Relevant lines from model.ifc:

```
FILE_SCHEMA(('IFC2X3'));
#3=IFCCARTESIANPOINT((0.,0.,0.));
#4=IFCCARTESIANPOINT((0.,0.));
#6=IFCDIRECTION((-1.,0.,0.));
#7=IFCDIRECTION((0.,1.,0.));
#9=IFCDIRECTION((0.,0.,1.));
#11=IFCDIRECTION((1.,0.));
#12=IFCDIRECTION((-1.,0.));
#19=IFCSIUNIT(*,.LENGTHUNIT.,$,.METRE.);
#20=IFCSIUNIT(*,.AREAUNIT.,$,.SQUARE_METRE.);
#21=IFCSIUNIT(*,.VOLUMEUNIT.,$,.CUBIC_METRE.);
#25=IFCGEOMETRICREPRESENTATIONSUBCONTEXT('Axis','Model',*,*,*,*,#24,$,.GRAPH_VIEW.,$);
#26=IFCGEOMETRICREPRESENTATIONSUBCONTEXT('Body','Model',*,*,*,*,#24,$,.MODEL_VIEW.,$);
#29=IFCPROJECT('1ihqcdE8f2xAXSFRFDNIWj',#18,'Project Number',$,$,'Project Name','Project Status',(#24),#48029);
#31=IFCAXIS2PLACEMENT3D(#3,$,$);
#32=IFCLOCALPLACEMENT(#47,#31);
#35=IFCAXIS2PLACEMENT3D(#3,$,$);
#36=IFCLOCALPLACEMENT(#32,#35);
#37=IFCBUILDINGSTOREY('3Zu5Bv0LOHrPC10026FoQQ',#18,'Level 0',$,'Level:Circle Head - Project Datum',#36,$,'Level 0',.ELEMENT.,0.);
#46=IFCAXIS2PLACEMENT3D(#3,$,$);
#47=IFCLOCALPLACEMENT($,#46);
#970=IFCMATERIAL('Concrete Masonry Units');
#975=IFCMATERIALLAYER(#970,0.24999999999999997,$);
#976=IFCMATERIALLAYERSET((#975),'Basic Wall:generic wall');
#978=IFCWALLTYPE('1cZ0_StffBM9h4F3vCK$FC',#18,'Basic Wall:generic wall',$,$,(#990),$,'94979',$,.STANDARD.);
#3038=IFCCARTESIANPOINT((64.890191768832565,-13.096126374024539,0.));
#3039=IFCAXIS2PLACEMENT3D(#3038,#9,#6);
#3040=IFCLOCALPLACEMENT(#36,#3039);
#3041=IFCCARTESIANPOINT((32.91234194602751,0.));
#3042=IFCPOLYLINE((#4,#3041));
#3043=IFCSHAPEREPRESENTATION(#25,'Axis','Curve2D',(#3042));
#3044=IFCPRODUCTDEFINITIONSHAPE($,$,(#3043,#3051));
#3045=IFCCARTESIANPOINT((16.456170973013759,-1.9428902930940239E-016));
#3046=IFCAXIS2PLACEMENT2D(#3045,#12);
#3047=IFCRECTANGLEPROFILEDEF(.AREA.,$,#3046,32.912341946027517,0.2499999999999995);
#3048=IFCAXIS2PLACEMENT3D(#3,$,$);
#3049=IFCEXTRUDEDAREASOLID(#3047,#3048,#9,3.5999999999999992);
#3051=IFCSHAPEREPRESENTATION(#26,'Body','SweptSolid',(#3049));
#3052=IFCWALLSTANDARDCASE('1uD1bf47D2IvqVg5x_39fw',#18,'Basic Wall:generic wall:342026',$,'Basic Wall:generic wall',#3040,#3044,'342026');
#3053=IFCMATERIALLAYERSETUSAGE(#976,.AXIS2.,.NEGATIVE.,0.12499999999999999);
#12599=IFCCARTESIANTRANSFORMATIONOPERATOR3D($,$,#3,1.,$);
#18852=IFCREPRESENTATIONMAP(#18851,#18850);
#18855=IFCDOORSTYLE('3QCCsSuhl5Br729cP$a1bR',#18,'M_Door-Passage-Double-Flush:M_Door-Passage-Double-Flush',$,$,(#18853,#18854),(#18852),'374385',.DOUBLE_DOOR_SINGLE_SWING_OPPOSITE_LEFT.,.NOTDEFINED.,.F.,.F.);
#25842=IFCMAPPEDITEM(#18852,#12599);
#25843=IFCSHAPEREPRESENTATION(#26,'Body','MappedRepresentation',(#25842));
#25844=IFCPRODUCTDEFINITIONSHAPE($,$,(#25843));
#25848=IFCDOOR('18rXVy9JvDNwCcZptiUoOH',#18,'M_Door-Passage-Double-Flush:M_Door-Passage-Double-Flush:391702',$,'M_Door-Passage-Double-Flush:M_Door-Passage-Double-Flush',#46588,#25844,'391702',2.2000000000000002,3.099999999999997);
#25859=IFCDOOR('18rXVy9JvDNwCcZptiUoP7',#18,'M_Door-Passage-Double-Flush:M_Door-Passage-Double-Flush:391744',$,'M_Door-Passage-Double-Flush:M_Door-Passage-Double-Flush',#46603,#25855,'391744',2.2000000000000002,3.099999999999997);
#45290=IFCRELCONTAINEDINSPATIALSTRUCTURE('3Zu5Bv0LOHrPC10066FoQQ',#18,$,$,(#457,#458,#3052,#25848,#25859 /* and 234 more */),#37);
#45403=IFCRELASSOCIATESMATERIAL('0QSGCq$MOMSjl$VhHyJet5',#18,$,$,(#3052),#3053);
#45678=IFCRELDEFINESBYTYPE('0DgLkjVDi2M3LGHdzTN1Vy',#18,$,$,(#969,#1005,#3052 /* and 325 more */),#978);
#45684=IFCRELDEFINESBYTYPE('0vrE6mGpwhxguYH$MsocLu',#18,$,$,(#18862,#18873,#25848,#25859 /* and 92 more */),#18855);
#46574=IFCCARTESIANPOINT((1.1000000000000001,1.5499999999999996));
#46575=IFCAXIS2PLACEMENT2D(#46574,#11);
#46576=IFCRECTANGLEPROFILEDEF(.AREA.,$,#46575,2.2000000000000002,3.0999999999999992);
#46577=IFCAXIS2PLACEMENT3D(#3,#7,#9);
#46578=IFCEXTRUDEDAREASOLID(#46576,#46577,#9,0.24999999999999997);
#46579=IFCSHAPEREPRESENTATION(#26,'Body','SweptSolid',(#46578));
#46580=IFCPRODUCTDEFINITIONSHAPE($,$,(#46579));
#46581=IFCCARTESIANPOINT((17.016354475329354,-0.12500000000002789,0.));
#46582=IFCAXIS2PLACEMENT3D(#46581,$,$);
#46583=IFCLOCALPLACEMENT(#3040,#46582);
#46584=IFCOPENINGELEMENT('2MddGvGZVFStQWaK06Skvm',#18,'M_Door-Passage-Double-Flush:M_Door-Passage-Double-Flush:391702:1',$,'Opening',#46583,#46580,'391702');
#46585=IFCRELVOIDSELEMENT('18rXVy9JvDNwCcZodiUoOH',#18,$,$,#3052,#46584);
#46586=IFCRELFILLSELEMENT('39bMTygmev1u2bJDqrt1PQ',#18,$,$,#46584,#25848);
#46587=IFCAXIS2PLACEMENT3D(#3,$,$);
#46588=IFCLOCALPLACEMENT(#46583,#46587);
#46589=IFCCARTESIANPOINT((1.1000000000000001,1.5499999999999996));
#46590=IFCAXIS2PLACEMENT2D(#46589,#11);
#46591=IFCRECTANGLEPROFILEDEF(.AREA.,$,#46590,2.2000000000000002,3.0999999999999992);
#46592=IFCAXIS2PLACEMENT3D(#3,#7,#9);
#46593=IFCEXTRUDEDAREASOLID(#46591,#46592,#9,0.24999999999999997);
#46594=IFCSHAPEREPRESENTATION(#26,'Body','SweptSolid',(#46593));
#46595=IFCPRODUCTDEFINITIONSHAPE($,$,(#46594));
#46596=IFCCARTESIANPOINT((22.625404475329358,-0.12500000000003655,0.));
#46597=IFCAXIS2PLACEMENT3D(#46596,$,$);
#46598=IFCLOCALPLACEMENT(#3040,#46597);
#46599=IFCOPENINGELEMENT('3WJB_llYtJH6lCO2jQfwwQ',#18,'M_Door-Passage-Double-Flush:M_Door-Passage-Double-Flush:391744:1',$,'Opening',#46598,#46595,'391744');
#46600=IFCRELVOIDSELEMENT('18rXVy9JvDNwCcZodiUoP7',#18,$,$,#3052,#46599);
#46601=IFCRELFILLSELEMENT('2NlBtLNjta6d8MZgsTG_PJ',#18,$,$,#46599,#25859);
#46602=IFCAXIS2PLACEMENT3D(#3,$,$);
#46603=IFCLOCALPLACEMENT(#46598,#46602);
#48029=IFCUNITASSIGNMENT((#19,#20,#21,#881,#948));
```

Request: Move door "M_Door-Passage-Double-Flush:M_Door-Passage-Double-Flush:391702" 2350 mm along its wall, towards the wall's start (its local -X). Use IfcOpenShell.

```python
import ifcopenshell
import ifcopenshell.api.geometry
import ifcopenshell.util.placement
import ifcopenshell.util.unit

model = ifcopenshell.open("model.ifc")
unit_scale = ifcopenshell.util.unit.calculate_unit_scale(model)

door = model.by_guid("18rXVy9JvDNwCcZptiUoOH")
opening = door.FillsVoids[0].RelatingOpeningElement
wall = opening.VoidsElements[0].RelatingBuildingElement

wall_matrix = ifcopenshell.util.placement.get_local_placement(wall.ObjectPlacement)
shift = wall_matrix[:3, 0] * -2.35 / unit_scale
before = ifcopenshell.util.placement.get_local_placement(door.ObjectPlacement)[:3, 3].copy()

# The door is placed relative to its opening, so it follows when the opening moves.
matrix = ifcopenshell.util.placement.get_local_placement(opening.ObjectPlacement)
matrix[:3, 3] += shift
ifcopenshell.api.geometry.edit_object_placement(
    model, product=opening, matrix=matrix, is_si=False, should_transform_children=True
)

after = ifcopenshell.util.placement.get_local_placement(door.ObjectPlacement)[:3, 3]
print("door moved by", (after - before).round(3) + 0.0)

model.write("model_rev.ifc")
```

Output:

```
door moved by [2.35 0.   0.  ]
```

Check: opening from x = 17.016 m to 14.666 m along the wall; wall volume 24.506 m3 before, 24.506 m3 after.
